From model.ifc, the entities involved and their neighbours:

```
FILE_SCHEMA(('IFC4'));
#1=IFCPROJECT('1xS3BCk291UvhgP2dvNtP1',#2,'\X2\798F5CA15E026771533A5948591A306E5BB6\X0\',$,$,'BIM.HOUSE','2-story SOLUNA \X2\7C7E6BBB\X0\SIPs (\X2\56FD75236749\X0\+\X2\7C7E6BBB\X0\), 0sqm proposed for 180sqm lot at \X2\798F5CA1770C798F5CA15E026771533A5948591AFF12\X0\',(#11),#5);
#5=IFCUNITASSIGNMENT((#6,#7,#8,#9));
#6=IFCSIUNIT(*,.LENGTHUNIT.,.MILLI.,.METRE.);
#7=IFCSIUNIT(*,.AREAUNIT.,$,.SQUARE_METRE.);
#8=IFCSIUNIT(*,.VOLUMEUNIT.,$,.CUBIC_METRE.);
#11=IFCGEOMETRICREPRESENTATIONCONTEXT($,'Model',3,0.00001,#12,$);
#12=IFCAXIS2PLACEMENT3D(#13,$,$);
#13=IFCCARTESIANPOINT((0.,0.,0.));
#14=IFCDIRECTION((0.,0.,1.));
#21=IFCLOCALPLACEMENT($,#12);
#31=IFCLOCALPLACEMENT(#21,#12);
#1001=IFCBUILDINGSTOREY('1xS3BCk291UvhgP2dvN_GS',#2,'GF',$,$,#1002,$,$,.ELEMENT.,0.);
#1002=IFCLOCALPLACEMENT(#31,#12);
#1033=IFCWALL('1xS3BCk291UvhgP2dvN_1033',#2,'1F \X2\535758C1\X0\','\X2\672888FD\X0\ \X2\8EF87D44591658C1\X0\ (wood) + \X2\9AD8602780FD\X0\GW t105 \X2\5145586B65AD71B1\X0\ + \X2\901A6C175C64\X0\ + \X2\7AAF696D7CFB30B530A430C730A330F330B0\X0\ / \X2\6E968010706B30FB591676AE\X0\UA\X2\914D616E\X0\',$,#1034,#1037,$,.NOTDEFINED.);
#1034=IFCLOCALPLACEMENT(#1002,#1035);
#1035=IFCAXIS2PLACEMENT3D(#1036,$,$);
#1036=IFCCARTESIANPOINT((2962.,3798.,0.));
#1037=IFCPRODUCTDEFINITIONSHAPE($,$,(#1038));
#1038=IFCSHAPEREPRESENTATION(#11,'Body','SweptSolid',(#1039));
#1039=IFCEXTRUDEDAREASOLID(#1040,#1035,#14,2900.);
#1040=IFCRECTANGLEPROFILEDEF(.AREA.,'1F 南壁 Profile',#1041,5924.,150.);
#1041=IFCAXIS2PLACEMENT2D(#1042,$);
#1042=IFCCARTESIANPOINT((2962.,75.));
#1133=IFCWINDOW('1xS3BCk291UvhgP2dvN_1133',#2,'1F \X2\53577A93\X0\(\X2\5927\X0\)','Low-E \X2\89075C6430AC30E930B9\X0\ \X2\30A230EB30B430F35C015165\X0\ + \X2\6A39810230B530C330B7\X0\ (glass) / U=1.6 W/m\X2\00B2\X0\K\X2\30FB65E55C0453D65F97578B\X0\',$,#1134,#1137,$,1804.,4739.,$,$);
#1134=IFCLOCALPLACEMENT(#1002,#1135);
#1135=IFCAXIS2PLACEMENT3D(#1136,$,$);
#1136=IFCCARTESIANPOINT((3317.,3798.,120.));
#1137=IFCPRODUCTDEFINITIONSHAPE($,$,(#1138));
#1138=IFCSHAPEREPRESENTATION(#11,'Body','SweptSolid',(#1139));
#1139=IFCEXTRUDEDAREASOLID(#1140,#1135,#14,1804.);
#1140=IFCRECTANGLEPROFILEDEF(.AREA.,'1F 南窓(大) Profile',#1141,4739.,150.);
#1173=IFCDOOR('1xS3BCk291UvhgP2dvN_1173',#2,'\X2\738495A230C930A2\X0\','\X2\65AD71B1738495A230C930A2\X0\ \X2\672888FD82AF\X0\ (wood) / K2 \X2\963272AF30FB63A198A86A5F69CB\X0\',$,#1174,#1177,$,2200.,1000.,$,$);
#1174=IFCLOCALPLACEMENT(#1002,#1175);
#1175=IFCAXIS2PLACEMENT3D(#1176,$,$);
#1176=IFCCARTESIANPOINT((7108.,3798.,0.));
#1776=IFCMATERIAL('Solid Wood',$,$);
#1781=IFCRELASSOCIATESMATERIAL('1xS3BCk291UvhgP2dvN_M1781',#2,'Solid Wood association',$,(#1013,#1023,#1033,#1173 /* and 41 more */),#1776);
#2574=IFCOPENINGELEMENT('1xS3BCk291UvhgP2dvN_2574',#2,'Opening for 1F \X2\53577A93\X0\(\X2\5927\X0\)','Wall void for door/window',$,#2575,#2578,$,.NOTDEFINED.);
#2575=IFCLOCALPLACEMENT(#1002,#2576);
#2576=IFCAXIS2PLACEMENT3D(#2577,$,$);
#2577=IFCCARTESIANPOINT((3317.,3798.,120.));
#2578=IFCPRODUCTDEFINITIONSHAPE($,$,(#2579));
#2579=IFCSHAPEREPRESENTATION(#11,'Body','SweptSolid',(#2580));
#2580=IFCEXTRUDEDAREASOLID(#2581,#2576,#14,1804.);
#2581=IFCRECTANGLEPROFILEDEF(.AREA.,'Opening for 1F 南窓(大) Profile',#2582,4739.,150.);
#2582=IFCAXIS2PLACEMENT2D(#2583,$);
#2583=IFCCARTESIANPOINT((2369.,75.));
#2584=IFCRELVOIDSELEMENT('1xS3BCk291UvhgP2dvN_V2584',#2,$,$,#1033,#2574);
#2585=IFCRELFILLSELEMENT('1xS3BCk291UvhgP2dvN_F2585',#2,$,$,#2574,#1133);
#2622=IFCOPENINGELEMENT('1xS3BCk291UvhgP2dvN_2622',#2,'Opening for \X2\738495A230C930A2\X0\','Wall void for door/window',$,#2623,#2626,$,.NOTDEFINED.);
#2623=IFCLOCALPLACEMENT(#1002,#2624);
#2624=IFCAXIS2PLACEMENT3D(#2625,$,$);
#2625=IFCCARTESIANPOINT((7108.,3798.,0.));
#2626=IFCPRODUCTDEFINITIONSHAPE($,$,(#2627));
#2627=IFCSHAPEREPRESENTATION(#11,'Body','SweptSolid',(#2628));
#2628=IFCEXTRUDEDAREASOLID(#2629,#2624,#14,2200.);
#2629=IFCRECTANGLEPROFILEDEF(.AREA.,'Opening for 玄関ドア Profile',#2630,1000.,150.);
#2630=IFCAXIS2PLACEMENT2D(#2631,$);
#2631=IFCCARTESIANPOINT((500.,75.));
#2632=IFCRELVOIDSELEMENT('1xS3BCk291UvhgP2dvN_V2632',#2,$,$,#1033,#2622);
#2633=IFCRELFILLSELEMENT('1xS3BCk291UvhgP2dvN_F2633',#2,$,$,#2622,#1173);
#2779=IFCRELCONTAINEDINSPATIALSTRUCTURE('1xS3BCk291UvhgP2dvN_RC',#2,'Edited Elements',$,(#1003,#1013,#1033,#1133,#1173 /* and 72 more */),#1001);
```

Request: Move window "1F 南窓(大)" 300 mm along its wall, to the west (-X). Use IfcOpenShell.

```python
import ifcopenshell
import ifcopenshell.api.geometry
import ifcopenshell.util.placement

model = ifcopenshell.open("model.ifc")

window = model.by_id(1133)
opening = window.FillsVoids[0].RelatingOpeningElement
wall = opening.VoidsElements[0].RelatingBuildingElement

wall_matrix = ifcopenshell.util.placement.get_local_placement(wall.ObjectPlacement)
shift = wall_matrix[:3, 0] * -300.0
before = ifcopenshell.util.placement.get_local_placement(window.ObjectPlacement)[:3, 3].copy()

# The window is not placed relative to its opening, so move both.
for product in (opening, window):
    matrix = ifcopenshell.util.placement.get_local_placement(product.ObjectPlacement)
    matrix[:3, 3] += shift
    ifcopenshell.api.geometry.edit_object_placement(model, product=product, matrix=matrix, is_si=False)

after = ifcopenshell.util.placement.get_local_placement(window.ObjectPlacement)[:3, 3]
print("window moved by", (after - before).round(3) + 0.0)

model.write("model_edited.ifc")
```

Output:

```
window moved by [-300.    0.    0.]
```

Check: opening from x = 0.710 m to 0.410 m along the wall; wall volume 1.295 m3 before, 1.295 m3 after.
